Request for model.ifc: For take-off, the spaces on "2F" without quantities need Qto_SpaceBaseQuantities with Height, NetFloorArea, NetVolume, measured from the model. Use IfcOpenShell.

First a look at what the model holds.

```python
import ifcopenshell
import ifcopenshell.util.element
import ifcopenshell.util.unit

model = ifcopenshell.open("model.ifc")
print(model.schema)
for unit_type in ("LENGTHUNIT", "AREAUNIT", "VOLUMEUNIT"):
    print(unit_type, ifcopenshell.util.unit.calculate_unit_scale(model, unit_type))
storey = next(s for s in model.by_type("IfcBuildingStorey") if s.Name == "2F")
spaces = [e for e in ifcopenshell.util.element.get_decomposition(storey) if e.is_a("IfcSpace")]
for e in sorted(spaces, key=lambda e: e.id()):
    print(e.id(), e.is_a(), e.Name, list(ifcopenshell.util.element.get_psets(e, qtos_only=True)), sep=" | ")
```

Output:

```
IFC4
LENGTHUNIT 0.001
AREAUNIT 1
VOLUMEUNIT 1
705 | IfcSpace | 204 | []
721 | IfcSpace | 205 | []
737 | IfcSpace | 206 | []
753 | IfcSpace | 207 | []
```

```python
import ifcopenshell
import ifcopenshell.api.pset
import ifcopenshell.geom
import ifcopenshell.util.element
import ifcopenshell.util.shape
import ifcopenshell.util.unit

model = ifcopenshell.open("model.ifc")
unit_scale = ifcopenshell.util.unit.calculate_unit_scale(model)
area_scale = ifcopenshell.util.unit.calculate_unit_scale(model, "AREAUNIT")
volume_scale = ifcopenshell.util.unit.calculate_unit_scale(model, "VOLUMEUNIT")
settings = ifcopenshell.geom.settings()

storey = next(s for s in model.by_type("IfcBuildingStorey") if s.Name == "2F")
spaces = [e for e in ifcopenshell.util.element.get_decomposition(storey) if e.is_a("IfcSpace")]

for e in sorted(spaces, key=lambda e: e.id()):
    if ifcopenshell.util.element.get_psets(e, qtos_only=True, should_inherit=False):
        continue
    # Geometry comes back in metres, in the element's own axes.
    shape = ifcopenshell.geom.create_shape(settings, e)
    values = {
        "Height": ifcopenshell.util.shape.get_z(shape.geometry) / unit_scale,
        "NetFloorArea": ifcopenshell.util.shape.get_footprint_area(shape.geometry) / area_scale,
        "NetVolume": ifcopenshell.util.shape.get_volume(shape.geometry) / volume_scale,
    }
    qto = ifcopenshell.api.pset.add_qto(model, product=e, name="Qto_SpaceBaseQuantities")
    ifcopenshell.api.pset.edit_qto(model, qto=qto, properties=values)
    print(e.id(), {k: round(v, 3) for k, v in values.items()})

model.write("model-out.ifc")
```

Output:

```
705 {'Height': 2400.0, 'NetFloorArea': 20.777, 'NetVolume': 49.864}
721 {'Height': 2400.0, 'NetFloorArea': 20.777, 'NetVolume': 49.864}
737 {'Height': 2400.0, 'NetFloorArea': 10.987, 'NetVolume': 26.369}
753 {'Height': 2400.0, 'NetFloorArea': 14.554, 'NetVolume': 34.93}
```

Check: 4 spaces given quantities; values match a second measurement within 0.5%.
